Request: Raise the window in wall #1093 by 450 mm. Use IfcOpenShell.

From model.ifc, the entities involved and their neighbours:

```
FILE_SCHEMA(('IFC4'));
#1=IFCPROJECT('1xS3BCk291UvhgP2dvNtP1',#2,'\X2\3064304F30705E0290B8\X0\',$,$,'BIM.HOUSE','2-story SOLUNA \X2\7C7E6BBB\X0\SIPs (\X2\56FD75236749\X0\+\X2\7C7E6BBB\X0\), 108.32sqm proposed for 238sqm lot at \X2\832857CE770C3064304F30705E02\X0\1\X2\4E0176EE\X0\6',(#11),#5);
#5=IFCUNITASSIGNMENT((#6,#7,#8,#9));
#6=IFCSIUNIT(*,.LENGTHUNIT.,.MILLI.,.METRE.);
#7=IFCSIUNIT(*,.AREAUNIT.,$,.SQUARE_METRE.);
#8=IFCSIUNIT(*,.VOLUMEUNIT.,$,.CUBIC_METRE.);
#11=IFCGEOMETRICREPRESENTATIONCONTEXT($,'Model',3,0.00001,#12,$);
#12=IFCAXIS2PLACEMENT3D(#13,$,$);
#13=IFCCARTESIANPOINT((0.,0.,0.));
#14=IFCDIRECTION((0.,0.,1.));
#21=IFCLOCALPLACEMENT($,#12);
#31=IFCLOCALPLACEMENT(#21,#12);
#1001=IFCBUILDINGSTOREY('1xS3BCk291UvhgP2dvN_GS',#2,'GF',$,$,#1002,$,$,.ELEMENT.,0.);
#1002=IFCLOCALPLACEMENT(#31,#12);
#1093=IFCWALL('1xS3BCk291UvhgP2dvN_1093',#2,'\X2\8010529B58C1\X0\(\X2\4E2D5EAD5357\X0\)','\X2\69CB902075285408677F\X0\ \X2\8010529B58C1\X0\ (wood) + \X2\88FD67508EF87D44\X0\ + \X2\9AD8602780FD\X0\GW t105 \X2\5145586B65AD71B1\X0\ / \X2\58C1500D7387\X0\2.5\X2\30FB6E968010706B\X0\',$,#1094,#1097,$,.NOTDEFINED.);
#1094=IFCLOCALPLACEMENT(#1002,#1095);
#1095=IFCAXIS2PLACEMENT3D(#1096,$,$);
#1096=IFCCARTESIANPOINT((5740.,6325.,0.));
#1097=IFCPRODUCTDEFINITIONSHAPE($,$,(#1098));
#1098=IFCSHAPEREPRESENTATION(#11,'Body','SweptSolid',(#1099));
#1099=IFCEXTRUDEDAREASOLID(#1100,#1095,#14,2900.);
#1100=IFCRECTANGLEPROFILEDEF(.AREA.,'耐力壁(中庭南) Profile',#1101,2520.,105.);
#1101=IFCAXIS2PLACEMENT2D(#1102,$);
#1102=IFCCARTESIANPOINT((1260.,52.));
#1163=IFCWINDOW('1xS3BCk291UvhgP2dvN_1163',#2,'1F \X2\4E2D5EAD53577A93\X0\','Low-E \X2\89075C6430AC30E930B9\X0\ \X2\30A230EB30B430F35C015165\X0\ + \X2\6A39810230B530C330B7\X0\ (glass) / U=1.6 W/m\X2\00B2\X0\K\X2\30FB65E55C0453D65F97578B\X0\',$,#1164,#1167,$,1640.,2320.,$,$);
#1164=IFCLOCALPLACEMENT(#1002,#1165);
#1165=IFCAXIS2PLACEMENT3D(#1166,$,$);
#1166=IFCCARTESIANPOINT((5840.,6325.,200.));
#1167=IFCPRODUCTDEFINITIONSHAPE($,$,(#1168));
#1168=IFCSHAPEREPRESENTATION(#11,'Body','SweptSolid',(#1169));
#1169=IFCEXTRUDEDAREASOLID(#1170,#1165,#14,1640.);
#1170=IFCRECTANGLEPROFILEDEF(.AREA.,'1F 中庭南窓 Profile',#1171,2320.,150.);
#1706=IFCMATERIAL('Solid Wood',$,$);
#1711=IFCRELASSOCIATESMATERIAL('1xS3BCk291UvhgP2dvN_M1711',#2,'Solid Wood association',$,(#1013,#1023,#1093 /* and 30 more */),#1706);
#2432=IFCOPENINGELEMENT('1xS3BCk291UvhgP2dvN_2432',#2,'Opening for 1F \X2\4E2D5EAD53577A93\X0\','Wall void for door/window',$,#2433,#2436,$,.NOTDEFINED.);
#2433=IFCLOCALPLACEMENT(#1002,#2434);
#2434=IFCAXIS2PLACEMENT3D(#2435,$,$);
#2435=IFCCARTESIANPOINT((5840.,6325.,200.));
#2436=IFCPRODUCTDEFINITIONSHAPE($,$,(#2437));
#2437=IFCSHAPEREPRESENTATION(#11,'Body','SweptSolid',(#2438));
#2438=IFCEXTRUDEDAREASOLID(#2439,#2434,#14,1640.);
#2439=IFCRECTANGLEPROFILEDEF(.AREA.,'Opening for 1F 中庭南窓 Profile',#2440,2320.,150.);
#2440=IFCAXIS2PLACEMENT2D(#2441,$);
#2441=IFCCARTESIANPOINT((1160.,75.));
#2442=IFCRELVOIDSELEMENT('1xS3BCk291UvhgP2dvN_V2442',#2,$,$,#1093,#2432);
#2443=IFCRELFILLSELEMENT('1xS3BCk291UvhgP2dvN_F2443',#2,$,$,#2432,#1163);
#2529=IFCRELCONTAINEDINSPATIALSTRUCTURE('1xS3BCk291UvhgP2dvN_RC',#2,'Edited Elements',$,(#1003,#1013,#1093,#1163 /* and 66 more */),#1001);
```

```python
import numpy as np
import ifcopenshell
import ifcopenshell.api.geometry
import ifcopenshell.util.placement
import ifcopenshell.util.unit

model = ifcopenshell.open("model.ifc")
unit_scale = ifcopenshell.util.unit.calculate_unit_scale(model)

window = model.by_guid("1xS3BCk291UvhgP2dvN_1163")
opening = window.FillsVoids[0].RelatingOpeningElement
dz = 450.0

shift = np.array([0.0, 0.0, dz])
# The window is not placed relative to its opening, so move both.
for product in (opening, window):
    matrix = ifcopenshell.util.placement.get_local_placement(product.ObjectPlacement)
    matrix[:3, 3] += shift
    ifcopenshell.api.geometry.edit_object_placement(model, product=product, matrix=matrix, is_si=False)

print(f"moved by {dz * unit_scale:+.3f} m")

model.write("model_edited.ifc")
```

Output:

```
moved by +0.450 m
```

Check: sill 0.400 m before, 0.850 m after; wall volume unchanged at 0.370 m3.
